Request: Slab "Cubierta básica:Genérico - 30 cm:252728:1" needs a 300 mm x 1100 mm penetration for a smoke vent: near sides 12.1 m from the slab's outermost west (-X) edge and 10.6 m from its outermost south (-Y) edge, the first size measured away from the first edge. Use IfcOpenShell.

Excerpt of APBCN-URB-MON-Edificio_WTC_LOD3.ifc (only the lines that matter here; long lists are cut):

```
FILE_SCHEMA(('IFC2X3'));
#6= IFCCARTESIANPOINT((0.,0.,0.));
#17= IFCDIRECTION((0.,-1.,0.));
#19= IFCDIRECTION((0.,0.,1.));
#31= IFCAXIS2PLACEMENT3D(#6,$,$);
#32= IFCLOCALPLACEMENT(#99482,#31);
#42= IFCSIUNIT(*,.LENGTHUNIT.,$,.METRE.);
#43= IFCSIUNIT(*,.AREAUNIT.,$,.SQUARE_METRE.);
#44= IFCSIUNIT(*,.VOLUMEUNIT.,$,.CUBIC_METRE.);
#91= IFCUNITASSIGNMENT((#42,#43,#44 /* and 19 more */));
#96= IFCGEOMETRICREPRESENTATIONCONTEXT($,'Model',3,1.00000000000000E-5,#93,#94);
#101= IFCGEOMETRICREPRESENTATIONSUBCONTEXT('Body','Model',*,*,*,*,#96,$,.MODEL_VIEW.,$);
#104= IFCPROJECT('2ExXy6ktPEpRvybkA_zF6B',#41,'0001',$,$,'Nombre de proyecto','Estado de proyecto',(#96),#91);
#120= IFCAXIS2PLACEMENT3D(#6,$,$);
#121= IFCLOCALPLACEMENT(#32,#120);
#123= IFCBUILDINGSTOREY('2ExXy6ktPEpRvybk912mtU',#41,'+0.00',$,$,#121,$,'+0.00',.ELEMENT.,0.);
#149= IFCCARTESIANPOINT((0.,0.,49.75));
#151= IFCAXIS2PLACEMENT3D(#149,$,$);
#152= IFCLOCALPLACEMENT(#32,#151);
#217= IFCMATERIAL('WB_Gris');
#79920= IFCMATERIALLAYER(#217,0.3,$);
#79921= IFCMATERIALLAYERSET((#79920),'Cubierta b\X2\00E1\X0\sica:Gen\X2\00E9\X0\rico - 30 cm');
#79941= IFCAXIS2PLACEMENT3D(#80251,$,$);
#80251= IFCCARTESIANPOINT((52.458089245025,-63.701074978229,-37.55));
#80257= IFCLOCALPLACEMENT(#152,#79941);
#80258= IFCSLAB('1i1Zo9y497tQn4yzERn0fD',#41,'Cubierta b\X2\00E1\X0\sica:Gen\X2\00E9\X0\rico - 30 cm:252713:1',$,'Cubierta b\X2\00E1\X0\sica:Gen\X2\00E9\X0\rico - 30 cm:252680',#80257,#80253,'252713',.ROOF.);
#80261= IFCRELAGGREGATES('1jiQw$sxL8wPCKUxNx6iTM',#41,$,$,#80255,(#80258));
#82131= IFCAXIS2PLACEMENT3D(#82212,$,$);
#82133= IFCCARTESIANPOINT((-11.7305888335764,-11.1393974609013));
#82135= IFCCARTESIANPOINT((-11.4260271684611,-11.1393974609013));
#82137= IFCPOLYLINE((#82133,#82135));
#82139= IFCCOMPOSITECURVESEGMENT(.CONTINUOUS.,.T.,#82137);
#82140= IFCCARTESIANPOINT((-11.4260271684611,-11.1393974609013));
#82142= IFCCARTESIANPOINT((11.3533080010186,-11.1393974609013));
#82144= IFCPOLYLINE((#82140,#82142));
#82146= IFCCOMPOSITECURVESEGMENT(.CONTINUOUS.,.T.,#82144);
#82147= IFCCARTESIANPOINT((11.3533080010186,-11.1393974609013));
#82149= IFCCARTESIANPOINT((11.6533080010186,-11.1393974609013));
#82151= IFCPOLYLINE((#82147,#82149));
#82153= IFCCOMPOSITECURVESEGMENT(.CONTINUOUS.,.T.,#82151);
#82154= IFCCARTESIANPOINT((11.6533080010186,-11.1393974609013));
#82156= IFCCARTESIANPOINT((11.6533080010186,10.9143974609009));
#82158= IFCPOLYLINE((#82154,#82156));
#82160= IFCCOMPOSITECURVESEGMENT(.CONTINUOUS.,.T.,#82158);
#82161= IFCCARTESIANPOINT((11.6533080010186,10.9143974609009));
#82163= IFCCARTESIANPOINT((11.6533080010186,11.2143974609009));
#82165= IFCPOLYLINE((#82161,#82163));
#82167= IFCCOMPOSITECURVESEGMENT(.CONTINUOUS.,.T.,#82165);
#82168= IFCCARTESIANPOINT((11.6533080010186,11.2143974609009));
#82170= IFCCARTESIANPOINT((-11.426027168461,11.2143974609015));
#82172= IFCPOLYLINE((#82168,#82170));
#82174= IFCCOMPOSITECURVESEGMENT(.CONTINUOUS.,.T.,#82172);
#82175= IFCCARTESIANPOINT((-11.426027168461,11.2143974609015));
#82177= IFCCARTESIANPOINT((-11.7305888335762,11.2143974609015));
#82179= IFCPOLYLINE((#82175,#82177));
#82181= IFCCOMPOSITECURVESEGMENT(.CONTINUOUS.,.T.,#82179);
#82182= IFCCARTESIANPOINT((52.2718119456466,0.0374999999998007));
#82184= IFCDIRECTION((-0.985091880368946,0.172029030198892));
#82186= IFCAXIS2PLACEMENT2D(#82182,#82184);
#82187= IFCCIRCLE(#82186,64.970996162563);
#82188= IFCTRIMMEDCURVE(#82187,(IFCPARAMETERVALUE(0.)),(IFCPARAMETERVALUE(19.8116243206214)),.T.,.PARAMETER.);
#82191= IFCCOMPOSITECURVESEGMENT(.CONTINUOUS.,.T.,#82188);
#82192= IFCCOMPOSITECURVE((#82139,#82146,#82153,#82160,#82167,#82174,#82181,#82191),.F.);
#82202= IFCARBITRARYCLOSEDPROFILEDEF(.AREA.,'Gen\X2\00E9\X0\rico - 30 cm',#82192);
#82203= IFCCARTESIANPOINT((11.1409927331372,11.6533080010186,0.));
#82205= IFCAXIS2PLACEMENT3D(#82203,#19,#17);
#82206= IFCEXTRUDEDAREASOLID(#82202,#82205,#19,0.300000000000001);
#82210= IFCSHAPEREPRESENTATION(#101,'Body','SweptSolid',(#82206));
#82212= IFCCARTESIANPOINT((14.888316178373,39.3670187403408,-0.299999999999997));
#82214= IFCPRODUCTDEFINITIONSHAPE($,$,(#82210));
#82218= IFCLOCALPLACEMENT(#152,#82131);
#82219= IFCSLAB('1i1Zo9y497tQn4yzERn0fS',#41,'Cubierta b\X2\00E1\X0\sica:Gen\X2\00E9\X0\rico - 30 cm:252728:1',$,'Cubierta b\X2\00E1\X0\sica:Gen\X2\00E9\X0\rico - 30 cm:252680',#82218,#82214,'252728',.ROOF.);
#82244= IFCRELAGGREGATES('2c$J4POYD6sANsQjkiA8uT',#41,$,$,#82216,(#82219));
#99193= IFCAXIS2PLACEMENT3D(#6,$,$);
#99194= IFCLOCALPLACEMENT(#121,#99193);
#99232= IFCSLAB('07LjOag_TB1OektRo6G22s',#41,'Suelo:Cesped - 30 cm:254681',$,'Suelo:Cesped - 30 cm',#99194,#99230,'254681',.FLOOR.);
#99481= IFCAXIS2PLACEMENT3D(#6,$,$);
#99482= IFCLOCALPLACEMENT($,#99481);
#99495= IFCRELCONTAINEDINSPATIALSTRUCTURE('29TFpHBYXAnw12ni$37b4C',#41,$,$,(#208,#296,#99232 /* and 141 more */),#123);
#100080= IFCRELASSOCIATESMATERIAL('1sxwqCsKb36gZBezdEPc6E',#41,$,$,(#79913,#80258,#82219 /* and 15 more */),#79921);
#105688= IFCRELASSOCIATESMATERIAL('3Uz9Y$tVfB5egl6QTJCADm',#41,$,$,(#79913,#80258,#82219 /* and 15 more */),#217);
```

```python
import numpy as np
import ifcopenshell
import ifcopenshell.api.feature
import ifcopenshell.api.geometry
import ifcopenshell.api.root
import ifcopenshell.geom
import ifcopenshell.util.placement
import ifcopenshell.util.representation
import ifcopenshell.util.shape
import ifcopenshell.util.unit

model = ifcopenshell.open("APBCN-URB-MON-Edificio_WTC_LOD3.ifc")
unit_scale = ifcopenshell.util.unit.calculate_unit_scale(model)
settings = ifcopenshell.geom.settings()


def volume(element):
    """Net volume in cubic metres, openings subtracted."""
    shape = ifcopenshell.geom.create_shape(settings, element)
    return ifcopenshell.util.shape.get_volume(shape.geometry)


slab = model.by_guid("1i1Zo9y497tQn4yzERn0fS")
before = volume(slab)

# Extent in the slab's own axes, in metres. The edges named are its -X and -Y sides.
slab_shape = ifcopenshell.geom.create_shape(settings, slab)
vertices = ifcopenshell.util.shape.get_vertices(slab_shape.geometry)
x_min, y_min, bottom = vertices.min(axis=0)
top = vertices[:, 2].max()

opening = ifcopenshell.api.root.create_entity(model, ifc_class="IfcOpeningElement", name="Smoke vent opening")
context = ifcopenshell.util.representation.get_context(model, "Model", "Body", "MODEL_VIEW")
width, depth = 0.3, 1.1
outline = [(0.0, 0.0), (width, 0.0), (width, depth), (0.0, depth), (0.0, 0.0)]
# Overshoot both faces by 50 mm so the cut is clean.
shape = ifcopenshell.api.geometry.add_slab_representation(
    model, context=context, depth=top - bottom + 0.1, polyline=outline
)
ifcopenshell.api.geometry.assign_representation(model, product=opening, representation=shape)

matrix = ifcopenshell.util.placement.get_local_placement(slab.ObjectPlacement)
matrix[:, 3] = matrix @ np.append(np.array([x_min + 12.1, y_min + 10.6, bottom - 0.05]) / unit_scale, 1.0)
ifcopenshell.api.geometry.edit_object_placement(model, product=opening, matrix=matrix, is_si=False)
ifcopenshell.api.feature.add_feature(model, feature=opening, element=slab)

after = volume(slab)

print(f"slab volume {before:.3f} -> {after:.3f} m3")

model.write("APBCN-URB-MON-Edificio_WTC_LOD3_v2.ifc")
```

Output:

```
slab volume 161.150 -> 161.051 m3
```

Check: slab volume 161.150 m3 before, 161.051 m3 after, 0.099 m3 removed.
